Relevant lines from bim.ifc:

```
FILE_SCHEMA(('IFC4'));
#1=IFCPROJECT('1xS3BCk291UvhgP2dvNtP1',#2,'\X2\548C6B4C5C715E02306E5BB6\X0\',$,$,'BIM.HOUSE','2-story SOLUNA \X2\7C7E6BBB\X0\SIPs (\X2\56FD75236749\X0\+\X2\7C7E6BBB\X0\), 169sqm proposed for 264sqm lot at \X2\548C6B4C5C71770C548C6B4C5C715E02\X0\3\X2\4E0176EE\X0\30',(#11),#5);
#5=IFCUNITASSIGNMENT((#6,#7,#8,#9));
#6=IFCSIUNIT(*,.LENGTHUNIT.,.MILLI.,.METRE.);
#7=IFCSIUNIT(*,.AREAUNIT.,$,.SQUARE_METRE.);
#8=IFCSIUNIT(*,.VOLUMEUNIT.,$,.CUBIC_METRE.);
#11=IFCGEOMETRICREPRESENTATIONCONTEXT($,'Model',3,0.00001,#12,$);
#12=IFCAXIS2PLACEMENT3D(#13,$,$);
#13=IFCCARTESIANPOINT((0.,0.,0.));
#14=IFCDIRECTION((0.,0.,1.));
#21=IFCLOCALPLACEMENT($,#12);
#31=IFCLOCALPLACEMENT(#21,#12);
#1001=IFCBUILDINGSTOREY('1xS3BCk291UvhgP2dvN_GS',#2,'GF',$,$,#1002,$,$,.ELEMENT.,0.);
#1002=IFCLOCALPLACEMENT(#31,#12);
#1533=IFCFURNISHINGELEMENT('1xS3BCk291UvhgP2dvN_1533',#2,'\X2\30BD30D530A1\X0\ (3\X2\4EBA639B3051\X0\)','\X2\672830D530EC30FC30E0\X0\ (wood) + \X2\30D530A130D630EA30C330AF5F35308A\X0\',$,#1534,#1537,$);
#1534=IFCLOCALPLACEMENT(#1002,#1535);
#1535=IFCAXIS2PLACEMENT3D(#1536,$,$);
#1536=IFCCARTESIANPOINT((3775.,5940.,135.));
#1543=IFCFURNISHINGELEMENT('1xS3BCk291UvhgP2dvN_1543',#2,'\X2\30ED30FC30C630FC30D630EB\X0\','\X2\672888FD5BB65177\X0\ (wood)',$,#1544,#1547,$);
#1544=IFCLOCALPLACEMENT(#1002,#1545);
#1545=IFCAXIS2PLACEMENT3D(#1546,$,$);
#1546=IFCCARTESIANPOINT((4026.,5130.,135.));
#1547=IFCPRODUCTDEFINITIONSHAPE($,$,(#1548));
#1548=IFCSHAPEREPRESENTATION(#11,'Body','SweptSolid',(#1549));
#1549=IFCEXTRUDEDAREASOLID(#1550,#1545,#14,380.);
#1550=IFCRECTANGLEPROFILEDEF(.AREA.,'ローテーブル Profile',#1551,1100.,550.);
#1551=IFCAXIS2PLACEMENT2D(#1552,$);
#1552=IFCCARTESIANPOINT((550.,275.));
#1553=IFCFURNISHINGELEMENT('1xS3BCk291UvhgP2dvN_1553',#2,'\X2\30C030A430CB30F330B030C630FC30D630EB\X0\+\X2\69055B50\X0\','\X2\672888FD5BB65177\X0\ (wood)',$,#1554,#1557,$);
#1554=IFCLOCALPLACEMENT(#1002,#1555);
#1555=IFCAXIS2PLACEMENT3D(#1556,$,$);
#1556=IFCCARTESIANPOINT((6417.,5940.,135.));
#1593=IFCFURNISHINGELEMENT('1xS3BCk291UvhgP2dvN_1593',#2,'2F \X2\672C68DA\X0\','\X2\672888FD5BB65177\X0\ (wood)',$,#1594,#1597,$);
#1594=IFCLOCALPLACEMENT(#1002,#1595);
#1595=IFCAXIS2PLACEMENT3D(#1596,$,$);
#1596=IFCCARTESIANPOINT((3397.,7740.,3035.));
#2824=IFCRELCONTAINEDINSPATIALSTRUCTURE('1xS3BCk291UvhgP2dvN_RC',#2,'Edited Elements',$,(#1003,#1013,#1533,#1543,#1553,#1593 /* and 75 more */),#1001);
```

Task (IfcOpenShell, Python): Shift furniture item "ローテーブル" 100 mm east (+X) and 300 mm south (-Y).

```python
import ifcopenshell
import ifcopenshell.api.geometry
import ifcopenshell.util.placement
import ifcopenshell.util.unit

model = ifcopenshell.open("bim.ifc")
unit_scale = ifcopenshell.util.unit.calculate_unit_scale(model)

item = model.by_guid("1xS3BCk291UvhgP2dvN_1543")
matrix = ifcopenshell.util.placement.get_local_placement(item.ObjectPlacement)
matrix[0, 3] += 0.1 / unit_scale
matrix[1, 3] -= 0.3 / unit_scale
ifcopenshell.api.geometry.edit_object_placement(model, product=item, matrix=matrix, is_si=False)

print(ifcopenshell.util.placement.get_local_placement(item.ObjectPlacement).round(3) + 0.0)

model.write("bim_edited.ifc")
```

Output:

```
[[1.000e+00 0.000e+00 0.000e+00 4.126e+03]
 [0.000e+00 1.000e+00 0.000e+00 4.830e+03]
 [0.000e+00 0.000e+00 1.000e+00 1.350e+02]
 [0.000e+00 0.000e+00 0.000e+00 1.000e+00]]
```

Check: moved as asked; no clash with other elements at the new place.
